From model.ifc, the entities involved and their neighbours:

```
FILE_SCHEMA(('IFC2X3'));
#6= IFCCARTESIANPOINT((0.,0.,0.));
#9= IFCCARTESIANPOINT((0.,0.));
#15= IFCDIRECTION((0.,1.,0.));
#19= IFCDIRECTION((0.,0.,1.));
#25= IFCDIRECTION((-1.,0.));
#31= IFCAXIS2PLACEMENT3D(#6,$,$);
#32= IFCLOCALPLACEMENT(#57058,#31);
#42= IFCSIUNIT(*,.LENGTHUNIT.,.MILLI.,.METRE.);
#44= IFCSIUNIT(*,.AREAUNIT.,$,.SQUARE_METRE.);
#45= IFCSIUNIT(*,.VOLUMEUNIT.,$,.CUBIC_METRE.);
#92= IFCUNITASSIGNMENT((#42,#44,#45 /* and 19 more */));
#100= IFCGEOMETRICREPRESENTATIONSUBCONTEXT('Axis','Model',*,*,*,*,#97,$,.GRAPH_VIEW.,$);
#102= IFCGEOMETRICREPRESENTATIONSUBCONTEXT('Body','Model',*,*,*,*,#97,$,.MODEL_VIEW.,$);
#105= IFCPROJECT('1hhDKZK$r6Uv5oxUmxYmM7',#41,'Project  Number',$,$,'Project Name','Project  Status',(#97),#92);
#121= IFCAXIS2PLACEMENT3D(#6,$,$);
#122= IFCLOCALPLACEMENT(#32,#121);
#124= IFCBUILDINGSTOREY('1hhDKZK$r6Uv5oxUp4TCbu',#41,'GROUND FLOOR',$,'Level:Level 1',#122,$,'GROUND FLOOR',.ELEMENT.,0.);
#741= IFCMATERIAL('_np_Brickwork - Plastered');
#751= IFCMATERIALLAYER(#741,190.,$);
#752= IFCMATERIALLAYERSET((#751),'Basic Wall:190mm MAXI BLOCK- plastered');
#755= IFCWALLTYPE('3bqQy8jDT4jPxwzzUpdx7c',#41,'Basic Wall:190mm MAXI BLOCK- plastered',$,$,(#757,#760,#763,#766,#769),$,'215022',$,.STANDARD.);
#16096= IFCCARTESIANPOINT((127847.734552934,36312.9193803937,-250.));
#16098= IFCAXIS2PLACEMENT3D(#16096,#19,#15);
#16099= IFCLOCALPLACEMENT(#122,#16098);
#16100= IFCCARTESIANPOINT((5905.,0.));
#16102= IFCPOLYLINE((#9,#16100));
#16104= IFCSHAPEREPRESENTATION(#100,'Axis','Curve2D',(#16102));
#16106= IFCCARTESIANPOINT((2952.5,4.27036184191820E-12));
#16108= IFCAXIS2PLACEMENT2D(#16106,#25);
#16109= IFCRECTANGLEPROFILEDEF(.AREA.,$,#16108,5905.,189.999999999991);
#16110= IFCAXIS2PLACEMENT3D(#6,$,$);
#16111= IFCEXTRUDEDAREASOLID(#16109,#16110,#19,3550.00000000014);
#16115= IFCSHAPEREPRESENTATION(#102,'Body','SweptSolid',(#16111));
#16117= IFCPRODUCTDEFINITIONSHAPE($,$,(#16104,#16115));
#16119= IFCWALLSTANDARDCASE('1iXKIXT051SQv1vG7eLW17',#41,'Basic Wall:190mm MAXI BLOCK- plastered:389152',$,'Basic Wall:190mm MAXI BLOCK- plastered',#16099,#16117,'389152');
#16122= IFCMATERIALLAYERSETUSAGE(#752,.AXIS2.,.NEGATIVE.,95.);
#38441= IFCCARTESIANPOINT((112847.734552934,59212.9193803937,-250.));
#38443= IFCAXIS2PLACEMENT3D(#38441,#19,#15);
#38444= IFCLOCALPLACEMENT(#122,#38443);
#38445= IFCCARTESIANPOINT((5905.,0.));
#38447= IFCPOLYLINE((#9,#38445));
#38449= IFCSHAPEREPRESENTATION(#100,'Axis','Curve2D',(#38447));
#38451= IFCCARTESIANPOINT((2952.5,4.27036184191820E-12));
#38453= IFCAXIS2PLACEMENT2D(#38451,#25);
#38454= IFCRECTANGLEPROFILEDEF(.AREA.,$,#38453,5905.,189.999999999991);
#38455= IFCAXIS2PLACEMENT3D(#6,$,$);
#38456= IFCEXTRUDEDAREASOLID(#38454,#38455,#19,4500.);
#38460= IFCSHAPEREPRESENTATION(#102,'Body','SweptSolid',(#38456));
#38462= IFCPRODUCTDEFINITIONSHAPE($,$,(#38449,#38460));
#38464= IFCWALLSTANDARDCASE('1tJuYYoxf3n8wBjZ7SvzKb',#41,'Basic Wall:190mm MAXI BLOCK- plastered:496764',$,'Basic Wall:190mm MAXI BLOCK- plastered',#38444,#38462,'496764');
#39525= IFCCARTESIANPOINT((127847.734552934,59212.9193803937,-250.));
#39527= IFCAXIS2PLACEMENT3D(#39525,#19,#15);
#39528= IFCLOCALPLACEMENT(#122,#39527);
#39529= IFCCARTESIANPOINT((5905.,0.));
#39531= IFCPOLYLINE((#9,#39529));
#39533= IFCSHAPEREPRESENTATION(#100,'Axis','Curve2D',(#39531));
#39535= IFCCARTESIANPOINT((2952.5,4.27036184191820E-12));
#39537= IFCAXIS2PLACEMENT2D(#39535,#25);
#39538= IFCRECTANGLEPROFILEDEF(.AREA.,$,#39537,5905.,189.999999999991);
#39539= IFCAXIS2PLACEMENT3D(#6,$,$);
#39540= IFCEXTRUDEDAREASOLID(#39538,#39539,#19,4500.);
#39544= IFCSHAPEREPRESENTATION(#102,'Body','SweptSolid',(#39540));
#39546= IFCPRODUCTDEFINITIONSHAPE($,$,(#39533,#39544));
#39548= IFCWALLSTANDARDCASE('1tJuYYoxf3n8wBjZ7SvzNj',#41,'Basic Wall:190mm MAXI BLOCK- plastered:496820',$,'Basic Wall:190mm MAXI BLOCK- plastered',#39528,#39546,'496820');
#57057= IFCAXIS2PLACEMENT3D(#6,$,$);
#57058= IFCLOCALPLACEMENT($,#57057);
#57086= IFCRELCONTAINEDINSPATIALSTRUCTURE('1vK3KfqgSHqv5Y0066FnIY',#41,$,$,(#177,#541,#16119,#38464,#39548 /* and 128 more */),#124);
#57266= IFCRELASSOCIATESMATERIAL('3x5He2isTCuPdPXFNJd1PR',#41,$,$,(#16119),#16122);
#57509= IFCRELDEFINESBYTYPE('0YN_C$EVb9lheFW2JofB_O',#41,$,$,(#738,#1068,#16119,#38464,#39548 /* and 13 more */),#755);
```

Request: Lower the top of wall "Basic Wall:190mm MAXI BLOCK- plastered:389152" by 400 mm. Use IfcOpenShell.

```python
import ifcopenshell
import ifcopenshell.geom
import ifcopenshell.util.representation
import ifcopenshell.util.shape
import ifcopenshell.util.unit

model = ifcopenshell.open("model.ifc")
unit_scale = ifcopenshell.util.unit.calculate_unit_scale(model)
settings = ifcopenshell.geom.settings()


def volume(element):
    """Net volume in cubic metres, openings subtracted."""
    shape = ifcopenshell.geom.create_shape(settings, element)
    return ifcopenshell.util.shape.get_volume(shape.geometry)


wall = model.by_guid("1iXKIXT051SQv1vG7eLW17")
before = volume(wall)

body = ifcopenshell.util.representation.get_representation(wall, "Model", "Body")
solid = body.Items[0]
old_height = solid.Depth
solid.Depth -= 0.4 / unit_scale
after = volume(wall)

print(f"height {old_height:g} -> {solid.Depth:g}, volume {before:.3f} -> {after:.3f} m3")

model.write("model-out.ifc")
```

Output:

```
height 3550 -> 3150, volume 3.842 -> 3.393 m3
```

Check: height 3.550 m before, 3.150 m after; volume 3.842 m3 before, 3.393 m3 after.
